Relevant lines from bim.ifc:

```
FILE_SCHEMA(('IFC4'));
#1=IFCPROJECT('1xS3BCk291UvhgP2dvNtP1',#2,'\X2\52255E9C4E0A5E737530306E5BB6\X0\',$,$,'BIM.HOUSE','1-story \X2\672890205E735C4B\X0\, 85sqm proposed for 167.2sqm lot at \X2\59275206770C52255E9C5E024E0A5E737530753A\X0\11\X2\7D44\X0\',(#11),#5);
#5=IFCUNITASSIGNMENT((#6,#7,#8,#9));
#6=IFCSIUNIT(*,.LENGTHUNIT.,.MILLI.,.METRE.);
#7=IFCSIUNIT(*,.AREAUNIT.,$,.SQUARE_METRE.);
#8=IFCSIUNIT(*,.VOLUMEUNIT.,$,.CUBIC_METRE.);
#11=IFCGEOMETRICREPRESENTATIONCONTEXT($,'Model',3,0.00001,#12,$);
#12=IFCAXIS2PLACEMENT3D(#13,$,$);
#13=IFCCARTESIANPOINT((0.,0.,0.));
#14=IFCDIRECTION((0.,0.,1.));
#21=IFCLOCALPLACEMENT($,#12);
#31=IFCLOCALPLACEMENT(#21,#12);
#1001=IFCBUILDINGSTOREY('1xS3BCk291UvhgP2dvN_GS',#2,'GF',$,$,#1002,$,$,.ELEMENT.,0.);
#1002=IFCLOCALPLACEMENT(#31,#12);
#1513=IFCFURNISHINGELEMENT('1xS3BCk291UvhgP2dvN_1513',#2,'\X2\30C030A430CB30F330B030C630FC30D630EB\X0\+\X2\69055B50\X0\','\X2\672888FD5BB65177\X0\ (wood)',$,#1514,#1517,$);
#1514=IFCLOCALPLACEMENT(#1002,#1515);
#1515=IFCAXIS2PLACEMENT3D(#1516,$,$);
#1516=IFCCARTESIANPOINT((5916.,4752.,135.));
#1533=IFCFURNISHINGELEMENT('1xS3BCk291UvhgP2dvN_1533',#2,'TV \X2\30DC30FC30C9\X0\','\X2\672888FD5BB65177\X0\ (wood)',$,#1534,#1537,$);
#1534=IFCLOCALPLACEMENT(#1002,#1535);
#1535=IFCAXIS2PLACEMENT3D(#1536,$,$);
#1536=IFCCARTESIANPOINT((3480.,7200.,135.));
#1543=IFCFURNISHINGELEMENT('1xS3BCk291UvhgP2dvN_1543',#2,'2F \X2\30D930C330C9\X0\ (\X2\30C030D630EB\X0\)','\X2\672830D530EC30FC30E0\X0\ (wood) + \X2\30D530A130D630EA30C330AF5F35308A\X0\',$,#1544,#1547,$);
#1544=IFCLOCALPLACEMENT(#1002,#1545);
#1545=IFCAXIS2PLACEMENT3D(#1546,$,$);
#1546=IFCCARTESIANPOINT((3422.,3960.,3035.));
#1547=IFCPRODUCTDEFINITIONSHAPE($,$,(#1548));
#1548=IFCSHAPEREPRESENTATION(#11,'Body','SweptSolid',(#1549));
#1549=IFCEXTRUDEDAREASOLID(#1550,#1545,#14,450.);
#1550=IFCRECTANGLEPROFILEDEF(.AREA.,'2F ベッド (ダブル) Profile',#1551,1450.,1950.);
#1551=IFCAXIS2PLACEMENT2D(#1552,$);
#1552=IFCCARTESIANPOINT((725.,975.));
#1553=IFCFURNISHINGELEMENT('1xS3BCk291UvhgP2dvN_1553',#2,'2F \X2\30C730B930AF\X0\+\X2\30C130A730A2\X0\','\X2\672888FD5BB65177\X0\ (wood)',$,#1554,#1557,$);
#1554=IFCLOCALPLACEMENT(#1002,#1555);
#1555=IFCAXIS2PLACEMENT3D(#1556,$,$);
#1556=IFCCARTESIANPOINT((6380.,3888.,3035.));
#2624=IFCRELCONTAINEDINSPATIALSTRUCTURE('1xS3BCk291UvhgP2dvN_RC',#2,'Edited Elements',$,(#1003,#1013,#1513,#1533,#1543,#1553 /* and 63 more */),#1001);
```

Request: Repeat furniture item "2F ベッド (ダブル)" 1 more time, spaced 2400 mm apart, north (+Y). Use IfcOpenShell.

```python
import numpy as np
import ifcopenshell
import ifcopenshell.api.geometry
import ifcopenshell.api.root
import ifcopenshell.util.element
import ifcopenshell.util.placement
import ifcopenshell.util.unit

model = ifcopenshell.open("bim.ifc")
unit_scale = ifcopenshell.util.unit.calculate_unit_scale(model)


def reuse_history(source, copy):
    """copy_class also copies each property set's owner history, people and application; keep the originals."""
    for rel in copy.IsDefinedBy:
        if rel.is_a("IfcRelDefinesByProperties") and (history := rel.RelatingPropertyDefinition.OwnerHistory):
            rel.RelatingPropertyDefinition.OwnerHistory = source.OwnerHistory
            ifcopenshell.util.element.remove_deep2(model, history)


source = model.by_guid("1xS3BCk291UvhgP2dvN_1543")
base = ifcopenshell.util.placement.get_local_placement(source.ObjectPlacement)
step = np.array([0.0, 1.0, 0.0]) * 2.4 / unit_scale

for i in range(1, 2):
    copy = ifcopenshell.api.root.copy_class(model, product=source)
    copy.Representation = ifcopenshell.util.element.copy_deep(
        model, source.Representation, exclude=["IfcGeometricRepresentationContext", "IfcRepresentationMap"]
    )
    reuse_history(source, copy)
    matrix = base.copy()
    matrix[:3, 3] += i * step
    print("added at", matrix[:3, 3].round(3) + 0.0)
    ifcopenshell.api.geometry.edit_object_placement(model, product=copy, matrix=matrix, is_si=False)

model.write("bim_rev.ifc")
```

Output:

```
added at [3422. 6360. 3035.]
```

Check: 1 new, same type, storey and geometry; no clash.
